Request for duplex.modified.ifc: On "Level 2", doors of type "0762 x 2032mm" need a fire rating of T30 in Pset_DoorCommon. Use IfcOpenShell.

First a look at what the model holds.

```python
import ifcopenshell
import ifcopenshell.util.element

model = ifcopenshell.open("duplex.modified.ifc")
print(model.schema)
storey = next(s for s in model.by_type("IfcBuildingStorey") if s.Name == "Level 2")
doors = [e for e in ifcopenshell.util.element.get_decomposition(storey) if e.is_a("IfcDoor")]
seen = {}
for e in doors:
    element_type = ifcopenshell.util.element.get_type(e)
    key = (element_type.Name if element_type != e and element_type else None, ifcopenshell.util.element.get_pset(e, "Pset_DoorCommon", "FireRating"))
    seen[key] = seen.get(key, 0) + 1
for (name, value), count in sorted(seen.items(), key=str):
    print(count, "x", name, "|", value)
```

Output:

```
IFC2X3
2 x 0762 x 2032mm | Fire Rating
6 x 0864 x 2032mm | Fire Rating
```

```python
import ifcopenshell
import ifcopenshell.api.pset
import ifcopenshell.util.element

model = ifcopenshell.open("duplex.modified.ifc")

storey = next(s for s in model.by_type("IfcBuildingStorey") if s.Name == "Level 2")
doors = [e for e in ifcopenshell.util.element.get_decomposition(storey) if e.is_a("IfcDoor")]

count = 0
for e in doors:
    element_type = ifcopenshell.util.element.get_type(e)
    if element_type in (None, e) or element_type.Name != "0762 x 2032mm":
        continue
    # add_pset returns the element's existing set when there is one.
    pset = ifcopenshell.api.pset.add_pset(model, product=e, name="Pset_DoorCommon")
    ifcopenshell.api.pset.edit_pset(model, pset=pset, properties={"FireRating": "T30"})
    count += 1

print(count, "doors updated")

model.write("duplex.modified_rev.ifc")
```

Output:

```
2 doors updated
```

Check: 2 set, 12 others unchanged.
